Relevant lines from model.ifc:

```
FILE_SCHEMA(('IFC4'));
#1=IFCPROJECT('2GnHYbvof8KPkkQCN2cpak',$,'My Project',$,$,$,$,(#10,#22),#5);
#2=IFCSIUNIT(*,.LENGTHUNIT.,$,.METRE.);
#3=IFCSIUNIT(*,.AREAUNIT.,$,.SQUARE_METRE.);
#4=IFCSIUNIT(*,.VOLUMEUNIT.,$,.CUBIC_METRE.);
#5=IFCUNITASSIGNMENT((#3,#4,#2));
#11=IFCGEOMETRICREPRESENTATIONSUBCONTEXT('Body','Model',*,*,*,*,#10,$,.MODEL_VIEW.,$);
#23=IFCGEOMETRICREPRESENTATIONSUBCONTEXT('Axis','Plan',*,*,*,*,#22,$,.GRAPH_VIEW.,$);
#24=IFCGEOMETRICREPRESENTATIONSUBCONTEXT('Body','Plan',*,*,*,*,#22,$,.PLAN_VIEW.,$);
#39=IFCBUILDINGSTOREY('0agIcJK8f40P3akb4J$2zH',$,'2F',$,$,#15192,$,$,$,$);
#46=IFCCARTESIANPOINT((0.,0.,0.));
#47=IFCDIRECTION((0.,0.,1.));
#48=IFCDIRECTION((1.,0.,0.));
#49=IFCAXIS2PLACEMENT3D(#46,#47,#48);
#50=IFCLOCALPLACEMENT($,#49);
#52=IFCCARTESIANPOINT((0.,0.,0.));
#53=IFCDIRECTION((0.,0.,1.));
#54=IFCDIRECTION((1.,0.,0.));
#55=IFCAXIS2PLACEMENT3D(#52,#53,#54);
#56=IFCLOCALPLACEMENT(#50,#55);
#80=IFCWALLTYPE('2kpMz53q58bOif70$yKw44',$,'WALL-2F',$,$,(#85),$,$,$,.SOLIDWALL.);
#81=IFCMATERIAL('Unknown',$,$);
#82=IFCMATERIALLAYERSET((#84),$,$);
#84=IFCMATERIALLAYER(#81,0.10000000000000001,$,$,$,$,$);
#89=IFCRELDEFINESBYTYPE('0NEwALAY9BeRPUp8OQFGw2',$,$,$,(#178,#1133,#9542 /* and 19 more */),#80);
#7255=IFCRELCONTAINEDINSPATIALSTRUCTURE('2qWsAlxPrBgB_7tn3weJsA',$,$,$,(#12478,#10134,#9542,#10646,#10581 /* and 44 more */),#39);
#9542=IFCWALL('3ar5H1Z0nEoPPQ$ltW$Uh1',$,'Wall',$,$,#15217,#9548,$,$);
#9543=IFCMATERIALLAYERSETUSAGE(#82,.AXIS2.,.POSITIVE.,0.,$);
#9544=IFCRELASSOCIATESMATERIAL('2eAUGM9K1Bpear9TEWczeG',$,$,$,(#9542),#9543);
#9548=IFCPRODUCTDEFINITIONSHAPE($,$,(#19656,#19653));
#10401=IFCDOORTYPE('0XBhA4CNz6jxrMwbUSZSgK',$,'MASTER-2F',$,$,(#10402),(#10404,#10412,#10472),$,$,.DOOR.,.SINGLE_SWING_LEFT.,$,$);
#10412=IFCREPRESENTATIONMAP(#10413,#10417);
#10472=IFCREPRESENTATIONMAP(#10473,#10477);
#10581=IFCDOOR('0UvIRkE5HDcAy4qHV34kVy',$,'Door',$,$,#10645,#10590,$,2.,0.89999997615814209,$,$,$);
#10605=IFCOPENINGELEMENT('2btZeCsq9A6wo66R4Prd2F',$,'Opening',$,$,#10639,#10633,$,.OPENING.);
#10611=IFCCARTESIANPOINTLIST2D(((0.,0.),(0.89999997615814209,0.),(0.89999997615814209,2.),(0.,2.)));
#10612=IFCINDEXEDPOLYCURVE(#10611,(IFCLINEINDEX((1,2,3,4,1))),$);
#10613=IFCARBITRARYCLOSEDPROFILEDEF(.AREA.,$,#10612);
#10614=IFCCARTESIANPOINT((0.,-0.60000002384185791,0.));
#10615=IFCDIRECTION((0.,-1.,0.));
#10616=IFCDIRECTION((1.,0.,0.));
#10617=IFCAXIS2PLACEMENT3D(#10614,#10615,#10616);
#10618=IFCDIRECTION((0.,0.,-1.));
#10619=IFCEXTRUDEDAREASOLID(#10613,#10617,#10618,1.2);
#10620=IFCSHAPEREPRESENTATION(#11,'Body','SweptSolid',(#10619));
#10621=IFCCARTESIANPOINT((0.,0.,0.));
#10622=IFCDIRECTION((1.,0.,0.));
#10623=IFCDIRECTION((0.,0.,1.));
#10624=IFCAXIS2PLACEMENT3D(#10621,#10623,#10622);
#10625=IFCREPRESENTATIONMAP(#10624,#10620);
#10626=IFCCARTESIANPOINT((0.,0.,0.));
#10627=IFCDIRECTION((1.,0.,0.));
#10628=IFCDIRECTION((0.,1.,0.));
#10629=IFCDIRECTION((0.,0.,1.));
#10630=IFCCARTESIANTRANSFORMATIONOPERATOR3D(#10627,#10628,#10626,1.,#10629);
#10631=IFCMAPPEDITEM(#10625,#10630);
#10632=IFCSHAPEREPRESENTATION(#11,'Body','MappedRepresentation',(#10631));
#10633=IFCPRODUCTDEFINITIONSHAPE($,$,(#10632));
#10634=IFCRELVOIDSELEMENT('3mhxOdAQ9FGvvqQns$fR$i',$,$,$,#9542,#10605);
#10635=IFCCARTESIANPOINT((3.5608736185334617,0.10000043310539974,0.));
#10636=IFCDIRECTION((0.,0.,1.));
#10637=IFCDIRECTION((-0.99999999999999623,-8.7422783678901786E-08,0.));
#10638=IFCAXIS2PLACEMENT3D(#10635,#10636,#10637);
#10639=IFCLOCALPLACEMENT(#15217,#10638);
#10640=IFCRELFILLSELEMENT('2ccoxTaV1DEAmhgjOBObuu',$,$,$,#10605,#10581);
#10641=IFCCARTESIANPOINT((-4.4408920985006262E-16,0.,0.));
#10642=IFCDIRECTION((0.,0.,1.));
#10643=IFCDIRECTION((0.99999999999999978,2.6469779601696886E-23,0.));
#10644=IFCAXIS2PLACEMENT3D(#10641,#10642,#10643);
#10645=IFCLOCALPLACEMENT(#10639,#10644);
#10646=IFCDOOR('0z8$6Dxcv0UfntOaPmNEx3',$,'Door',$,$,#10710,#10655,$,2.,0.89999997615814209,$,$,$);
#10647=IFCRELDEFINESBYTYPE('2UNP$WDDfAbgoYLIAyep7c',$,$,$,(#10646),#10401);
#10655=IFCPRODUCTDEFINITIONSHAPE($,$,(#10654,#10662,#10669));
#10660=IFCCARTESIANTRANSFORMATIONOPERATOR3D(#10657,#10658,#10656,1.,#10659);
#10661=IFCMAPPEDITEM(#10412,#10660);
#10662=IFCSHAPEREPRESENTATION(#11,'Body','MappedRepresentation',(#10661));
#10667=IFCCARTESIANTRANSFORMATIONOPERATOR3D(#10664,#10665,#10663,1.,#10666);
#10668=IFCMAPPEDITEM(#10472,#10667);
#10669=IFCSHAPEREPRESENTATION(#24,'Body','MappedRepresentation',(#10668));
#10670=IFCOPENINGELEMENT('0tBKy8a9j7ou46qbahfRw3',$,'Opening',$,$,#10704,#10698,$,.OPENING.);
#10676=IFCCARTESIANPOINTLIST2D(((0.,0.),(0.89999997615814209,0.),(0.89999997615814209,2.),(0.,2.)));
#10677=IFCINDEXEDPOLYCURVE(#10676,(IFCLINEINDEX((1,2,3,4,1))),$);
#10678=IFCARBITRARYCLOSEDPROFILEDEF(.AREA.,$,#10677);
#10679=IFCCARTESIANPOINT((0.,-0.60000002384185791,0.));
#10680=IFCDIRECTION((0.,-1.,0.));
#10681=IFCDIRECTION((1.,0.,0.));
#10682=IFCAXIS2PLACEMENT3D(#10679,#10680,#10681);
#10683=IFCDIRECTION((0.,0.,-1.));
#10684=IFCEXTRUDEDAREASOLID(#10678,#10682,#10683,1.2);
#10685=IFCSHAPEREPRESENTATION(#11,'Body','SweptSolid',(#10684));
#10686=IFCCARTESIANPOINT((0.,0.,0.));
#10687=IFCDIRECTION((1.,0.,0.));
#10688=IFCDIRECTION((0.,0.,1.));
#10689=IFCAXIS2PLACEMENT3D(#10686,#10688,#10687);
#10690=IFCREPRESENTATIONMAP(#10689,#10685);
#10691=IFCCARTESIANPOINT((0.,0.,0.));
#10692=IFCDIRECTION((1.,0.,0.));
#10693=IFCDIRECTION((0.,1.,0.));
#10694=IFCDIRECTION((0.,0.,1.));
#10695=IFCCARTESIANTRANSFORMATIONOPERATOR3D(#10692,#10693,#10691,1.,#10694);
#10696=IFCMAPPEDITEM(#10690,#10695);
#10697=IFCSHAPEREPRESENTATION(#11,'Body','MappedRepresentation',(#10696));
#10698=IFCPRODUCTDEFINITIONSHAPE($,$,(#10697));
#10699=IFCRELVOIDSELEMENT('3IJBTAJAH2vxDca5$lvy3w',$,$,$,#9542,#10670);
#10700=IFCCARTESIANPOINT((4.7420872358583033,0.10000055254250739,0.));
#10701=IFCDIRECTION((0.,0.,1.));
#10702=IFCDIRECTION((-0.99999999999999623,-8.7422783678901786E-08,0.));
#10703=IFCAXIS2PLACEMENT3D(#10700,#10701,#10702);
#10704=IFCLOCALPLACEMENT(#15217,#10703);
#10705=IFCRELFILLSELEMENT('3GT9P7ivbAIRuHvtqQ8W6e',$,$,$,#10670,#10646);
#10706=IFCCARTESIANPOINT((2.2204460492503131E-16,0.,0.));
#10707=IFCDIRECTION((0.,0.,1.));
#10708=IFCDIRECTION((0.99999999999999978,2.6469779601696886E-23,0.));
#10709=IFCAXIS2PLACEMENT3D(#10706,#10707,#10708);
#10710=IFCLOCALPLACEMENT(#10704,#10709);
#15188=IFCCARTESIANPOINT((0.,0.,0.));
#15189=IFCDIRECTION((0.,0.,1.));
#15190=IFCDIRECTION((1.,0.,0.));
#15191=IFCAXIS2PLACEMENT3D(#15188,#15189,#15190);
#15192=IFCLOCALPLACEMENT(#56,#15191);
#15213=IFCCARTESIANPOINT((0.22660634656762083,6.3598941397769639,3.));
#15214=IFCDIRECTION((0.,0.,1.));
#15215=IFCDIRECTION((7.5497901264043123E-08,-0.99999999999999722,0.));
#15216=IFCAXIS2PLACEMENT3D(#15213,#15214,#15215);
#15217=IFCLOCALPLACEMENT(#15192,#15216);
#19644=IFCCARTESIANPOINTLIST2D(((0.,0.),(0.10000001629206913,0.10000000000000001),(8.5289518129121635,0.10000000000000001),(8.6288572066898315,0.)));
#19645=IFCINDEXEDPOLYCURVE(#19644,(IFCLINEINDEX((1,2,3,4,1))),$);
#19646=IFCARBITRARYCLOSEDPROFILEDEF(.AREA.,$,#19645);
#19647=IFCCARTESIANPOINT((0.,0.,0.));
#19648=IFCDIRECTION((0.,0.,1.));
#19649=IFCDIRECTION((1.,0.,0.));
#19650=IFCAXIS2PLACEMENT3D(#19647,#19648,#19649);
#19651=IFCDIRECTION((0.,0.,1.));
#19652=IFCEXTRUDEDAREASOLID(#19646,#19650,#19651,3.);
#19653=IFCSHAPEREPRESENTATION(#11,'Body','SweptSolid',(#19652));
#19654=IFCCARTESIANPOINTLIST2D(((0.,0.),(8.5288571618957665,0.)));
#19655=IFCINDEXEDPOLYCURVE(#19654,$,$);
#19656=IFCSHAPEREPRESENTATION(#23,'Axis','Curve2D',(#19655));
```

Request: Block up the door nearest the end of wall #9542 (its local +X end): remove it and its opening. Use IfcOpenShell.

```python
import ifcopenshell
import ifcopenshell.api.feature
import ifcopenshell.api.root
import ifcopenshell.geom
import ifcopenshell.util.shape

model = ifcopenshell.open("model.ifc")
settings = ifcopenshell.geom.settings()


def volume(element):
    """Net volume in cubic metres, openings subtracted."""
    shape = ifcopenshell.geom.create_shape(settings, element)
    return ifcopenshell.util.shape.get_volume(shape.geometry)


door = model.by_guid("0z8$6Dxcv0UfntOaPmNEx3")
opening = door.FillsVoids[0].RelatingOpeningElement
wall = opening.VoidsElements[0].RelatingBuildingElement
before = volume(wall)

ifcopenshell.api.root.remove_product(model, product=door)
ifcopenshell.api.feature.remove_feature(model, feature=opening)

after = volume(wall)

print(f"wall volume {before:.3f} -> {after:.3f} m3")

model.write("model-out.ifc")
```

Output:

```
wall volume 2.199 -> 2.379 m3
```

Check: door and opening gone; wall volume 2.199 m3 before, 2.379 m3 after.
